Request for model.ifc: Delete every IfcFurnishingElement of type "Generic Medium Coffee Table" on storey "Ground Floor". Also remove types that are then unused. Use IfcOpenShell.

First a look at what the model holds.

```python
import ifcopenshell
import ifcopenshell.util.element

model = ifcopenshell.open("model.ifc")
print(model.schema)
storey = next(s for s in model.by_type("IfcBuildingStorey") if s.Name == "Ground Floor")
furniture = [e for e in ifcopenshell.util.element.get_decomposition(storey) if e.is_a("IfcFurnishingElement")]
seen = {}
for e in furniture:
    element_type = ifcopenshell.util.element.get_type(e)
    name = element_type.Name if element_type not in (None, e) else None
    seen[name] = seen.get(name, 0) + 1
for name, count in sorted(seen.items(), key=str):
    print(count, "x", name)
```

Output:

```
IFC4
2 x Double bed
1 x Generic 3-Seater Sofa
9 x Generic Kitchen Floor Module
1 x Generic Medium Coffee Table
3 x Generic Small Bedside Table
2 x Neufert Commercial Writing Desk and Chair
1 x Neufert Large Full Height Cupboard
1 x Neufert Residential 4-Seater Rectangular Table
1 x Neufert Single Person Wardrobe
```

```python
import ifcopenshell
import ifcopenshell.api.root
import ifcopenshell.util.element

model = ifcopenshell.open("model.ifc")

storey = next(s for s in model.by_type("IfcBuildingStorey") if s.Name == "Ground Floor")
furniture = [e for e in ifcopenshell.util.element.get_decomposition(storey) if e.is_a("IfcFurnishingElement")]
targets = [e for e in furniture if (t := ifcopenshell.util.element.get_type(e)) not in (None, e) and t.Name == "Generic Medium Coffee Table"]
types = {ifcopenshell.util.element.get_type(e) for e in targets} - {None, *targets}

for e in targets:
    ifcopenshell.api.root.remove_product(model, product=e)
print(len(targets), "removed")

unused = [t for t in types if not ifcopenshell.util.element.get_types(t)]
for t in unused:
    ifcopenshell.api.root.remove_product(model, product=t)
print(len(unused), "unused types removed")

model.write("model-out.ifc")
```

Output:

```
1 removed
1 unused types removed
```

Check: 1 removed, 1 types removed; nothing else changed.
